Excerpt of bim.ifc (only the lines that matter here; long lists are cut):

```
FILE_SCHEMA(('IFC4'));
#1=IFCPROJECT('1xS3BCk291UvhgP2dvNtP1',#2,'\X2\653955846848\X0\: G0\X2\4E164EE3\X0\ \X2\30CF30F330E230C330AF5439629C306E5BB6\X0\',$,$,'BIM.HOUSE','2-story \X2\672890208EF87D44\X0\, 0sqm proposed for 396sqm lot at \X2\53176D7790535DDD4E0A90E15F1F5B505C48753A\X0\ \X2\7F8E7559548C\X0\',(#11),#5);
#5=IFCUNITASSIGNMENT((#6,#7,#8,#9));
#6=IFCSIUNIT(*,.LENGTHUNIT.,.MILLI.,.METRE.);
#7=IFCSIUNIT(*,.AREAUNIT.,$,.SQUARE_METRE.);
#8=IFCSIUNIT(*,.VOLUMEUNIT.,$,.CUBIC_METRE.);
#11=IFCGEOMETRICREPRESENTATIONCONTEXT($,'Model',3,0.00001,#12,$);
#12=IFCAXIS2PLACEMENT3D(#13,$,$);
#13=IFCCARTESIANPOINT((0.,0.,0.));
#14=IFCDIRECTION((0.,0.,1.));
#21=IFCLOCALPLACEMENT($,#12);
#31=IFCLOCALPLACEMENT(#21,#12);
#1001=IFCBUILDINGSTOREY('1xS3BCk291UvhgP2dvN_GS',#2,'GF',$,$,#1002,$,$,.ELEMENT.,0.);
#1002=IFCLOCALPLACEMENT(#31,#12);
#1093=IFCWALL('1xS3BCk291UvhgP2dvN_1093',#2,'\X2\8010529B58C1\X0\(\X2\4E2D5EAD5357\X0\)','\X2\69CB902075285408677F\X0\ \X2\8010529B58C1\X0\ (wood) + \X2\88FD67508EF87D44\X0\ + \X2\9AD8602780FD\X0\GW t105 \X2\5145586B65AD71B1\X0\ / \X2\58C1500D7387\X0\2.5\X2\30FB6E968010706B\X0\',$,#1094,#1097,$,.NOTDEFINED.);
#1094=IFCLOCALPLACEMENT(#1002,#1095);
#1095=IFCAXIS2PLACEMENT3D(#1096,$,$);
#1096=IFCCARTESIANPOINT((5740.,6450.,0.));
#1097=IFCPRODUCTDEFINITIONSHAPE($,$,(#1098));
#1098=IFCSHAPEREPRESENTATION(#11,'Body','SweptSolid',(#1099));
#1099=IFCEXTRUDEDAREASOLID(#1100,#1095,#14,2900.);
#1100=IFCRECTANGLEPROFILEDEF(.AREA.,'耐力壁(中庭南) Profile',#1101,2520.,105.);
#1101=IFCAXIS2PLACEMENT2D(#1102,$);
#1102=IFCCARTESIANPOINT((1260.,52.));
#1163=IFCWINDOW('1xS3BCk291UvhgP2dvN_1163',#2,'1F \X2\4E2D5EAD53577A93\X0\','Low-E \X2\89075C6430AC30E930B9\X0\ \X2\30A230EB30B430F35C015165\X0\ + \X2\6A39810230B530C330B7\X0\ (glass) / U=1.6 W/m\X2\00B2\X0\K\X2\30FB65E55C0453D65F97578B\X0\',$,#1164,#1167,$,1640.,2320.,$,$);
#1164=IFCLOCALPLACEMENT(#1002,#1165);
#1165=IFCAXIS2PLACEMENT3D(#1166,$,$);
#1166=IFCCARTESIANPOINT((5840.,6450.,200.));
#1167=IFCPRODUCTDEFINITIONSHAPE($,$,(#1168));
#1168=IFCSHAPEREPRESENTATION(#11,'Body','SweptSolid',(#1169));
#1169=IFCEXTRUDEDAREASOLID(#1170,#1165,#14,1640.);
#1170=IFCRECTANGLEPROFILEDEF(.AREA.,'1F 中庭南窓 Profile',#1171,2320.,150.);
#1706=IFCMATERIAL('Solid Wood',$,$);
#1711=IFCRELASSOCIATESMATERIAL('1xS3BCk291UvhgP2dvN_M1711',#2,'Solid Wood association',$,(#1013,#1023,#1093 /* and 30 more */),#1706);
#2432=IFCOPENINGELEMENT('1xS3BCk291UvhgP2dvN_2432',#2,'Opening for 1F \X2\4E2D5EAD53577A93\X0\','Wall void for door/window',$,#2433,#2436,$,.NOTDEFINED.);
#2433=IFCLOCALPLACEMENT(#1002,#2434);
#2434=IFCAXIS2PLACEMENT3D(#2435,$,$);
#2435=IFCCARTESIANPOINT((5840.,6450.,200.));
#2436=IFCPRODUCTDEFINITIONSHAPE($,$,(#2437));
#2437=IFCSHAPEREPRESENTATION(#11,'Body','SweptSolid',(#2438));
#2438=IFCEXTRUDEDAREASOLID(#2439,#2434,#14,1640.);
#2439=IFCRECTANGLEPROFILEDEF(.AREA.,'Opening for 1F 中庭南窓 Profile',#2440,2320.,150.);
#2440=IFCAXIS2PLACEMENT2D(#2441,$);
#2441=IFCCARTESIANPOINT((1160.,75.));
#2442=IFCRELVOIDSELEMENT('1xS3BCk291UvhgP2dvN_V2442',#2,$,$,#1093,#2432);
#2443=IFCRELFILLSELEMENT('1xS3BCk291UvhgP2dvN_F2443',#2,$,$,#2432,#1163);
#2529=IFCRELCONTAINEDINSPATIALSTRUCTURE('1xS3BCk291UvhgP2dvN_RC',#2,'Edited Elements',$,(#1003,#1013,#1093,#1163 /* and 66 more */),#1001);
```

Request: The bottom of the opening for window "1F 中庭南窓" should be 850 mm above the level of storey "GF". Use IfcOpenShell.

```python
import numpy as np
import ifcopenshell
import ifcopenshell.api.geometry
import ifcopenshell.geom
import ifcopenshell.util.element
import ifcopenshell.util.placement
import ifcopenshell.util.shape
import ifcopenshell.util.unit

model = ifcopenshell.open("bim.ifc")
unit_scale = ifcopenshell.util.unit.calculate_unit_scale(model)

window = model.by_guid("1xS3BCk291UvhgP2dvN_1163")
opening = window.FillsVoids[0].RelatingOpeningElement
storey = ifcopenshell.util.element.get_container(window, ifc_class="IfcBuildingStorey")
level = ifcopenshell.util.placement.get_local_placement(storey.ObjectPlacement)[2, 3]

# The opening's origin need not be at the sill, so measure its lowest point.
shape = ifcopenshell.geom.create_shape(ifcopenshell.geom.settings(), opening)
bottom = ifcopenshell.util.shape.get_shape_bottom_elevation(shape, shape.geometry) / unit_scale
dz = level + 850.0 - bottom

shift = np.array([0.0, 0.0, dz])
# The window is not placed relative to its opening, so move both.
for product in (opening, window):
    matrix = ifcopenshell.util.placement.get_local_placement(product.ObjectPlacement)
    matrix[:3, 3] += shift
    ifcopenshell.api.geometry.edit_object_placement(model, product=product, matrix=matrix, is_si=False)

print(f"moved by {dz * unit_scale:+.3f} m")

model.write("bim-out.ifc")
```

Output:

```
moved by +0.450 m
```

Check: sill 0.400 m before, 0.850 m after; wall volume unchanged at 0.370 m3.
